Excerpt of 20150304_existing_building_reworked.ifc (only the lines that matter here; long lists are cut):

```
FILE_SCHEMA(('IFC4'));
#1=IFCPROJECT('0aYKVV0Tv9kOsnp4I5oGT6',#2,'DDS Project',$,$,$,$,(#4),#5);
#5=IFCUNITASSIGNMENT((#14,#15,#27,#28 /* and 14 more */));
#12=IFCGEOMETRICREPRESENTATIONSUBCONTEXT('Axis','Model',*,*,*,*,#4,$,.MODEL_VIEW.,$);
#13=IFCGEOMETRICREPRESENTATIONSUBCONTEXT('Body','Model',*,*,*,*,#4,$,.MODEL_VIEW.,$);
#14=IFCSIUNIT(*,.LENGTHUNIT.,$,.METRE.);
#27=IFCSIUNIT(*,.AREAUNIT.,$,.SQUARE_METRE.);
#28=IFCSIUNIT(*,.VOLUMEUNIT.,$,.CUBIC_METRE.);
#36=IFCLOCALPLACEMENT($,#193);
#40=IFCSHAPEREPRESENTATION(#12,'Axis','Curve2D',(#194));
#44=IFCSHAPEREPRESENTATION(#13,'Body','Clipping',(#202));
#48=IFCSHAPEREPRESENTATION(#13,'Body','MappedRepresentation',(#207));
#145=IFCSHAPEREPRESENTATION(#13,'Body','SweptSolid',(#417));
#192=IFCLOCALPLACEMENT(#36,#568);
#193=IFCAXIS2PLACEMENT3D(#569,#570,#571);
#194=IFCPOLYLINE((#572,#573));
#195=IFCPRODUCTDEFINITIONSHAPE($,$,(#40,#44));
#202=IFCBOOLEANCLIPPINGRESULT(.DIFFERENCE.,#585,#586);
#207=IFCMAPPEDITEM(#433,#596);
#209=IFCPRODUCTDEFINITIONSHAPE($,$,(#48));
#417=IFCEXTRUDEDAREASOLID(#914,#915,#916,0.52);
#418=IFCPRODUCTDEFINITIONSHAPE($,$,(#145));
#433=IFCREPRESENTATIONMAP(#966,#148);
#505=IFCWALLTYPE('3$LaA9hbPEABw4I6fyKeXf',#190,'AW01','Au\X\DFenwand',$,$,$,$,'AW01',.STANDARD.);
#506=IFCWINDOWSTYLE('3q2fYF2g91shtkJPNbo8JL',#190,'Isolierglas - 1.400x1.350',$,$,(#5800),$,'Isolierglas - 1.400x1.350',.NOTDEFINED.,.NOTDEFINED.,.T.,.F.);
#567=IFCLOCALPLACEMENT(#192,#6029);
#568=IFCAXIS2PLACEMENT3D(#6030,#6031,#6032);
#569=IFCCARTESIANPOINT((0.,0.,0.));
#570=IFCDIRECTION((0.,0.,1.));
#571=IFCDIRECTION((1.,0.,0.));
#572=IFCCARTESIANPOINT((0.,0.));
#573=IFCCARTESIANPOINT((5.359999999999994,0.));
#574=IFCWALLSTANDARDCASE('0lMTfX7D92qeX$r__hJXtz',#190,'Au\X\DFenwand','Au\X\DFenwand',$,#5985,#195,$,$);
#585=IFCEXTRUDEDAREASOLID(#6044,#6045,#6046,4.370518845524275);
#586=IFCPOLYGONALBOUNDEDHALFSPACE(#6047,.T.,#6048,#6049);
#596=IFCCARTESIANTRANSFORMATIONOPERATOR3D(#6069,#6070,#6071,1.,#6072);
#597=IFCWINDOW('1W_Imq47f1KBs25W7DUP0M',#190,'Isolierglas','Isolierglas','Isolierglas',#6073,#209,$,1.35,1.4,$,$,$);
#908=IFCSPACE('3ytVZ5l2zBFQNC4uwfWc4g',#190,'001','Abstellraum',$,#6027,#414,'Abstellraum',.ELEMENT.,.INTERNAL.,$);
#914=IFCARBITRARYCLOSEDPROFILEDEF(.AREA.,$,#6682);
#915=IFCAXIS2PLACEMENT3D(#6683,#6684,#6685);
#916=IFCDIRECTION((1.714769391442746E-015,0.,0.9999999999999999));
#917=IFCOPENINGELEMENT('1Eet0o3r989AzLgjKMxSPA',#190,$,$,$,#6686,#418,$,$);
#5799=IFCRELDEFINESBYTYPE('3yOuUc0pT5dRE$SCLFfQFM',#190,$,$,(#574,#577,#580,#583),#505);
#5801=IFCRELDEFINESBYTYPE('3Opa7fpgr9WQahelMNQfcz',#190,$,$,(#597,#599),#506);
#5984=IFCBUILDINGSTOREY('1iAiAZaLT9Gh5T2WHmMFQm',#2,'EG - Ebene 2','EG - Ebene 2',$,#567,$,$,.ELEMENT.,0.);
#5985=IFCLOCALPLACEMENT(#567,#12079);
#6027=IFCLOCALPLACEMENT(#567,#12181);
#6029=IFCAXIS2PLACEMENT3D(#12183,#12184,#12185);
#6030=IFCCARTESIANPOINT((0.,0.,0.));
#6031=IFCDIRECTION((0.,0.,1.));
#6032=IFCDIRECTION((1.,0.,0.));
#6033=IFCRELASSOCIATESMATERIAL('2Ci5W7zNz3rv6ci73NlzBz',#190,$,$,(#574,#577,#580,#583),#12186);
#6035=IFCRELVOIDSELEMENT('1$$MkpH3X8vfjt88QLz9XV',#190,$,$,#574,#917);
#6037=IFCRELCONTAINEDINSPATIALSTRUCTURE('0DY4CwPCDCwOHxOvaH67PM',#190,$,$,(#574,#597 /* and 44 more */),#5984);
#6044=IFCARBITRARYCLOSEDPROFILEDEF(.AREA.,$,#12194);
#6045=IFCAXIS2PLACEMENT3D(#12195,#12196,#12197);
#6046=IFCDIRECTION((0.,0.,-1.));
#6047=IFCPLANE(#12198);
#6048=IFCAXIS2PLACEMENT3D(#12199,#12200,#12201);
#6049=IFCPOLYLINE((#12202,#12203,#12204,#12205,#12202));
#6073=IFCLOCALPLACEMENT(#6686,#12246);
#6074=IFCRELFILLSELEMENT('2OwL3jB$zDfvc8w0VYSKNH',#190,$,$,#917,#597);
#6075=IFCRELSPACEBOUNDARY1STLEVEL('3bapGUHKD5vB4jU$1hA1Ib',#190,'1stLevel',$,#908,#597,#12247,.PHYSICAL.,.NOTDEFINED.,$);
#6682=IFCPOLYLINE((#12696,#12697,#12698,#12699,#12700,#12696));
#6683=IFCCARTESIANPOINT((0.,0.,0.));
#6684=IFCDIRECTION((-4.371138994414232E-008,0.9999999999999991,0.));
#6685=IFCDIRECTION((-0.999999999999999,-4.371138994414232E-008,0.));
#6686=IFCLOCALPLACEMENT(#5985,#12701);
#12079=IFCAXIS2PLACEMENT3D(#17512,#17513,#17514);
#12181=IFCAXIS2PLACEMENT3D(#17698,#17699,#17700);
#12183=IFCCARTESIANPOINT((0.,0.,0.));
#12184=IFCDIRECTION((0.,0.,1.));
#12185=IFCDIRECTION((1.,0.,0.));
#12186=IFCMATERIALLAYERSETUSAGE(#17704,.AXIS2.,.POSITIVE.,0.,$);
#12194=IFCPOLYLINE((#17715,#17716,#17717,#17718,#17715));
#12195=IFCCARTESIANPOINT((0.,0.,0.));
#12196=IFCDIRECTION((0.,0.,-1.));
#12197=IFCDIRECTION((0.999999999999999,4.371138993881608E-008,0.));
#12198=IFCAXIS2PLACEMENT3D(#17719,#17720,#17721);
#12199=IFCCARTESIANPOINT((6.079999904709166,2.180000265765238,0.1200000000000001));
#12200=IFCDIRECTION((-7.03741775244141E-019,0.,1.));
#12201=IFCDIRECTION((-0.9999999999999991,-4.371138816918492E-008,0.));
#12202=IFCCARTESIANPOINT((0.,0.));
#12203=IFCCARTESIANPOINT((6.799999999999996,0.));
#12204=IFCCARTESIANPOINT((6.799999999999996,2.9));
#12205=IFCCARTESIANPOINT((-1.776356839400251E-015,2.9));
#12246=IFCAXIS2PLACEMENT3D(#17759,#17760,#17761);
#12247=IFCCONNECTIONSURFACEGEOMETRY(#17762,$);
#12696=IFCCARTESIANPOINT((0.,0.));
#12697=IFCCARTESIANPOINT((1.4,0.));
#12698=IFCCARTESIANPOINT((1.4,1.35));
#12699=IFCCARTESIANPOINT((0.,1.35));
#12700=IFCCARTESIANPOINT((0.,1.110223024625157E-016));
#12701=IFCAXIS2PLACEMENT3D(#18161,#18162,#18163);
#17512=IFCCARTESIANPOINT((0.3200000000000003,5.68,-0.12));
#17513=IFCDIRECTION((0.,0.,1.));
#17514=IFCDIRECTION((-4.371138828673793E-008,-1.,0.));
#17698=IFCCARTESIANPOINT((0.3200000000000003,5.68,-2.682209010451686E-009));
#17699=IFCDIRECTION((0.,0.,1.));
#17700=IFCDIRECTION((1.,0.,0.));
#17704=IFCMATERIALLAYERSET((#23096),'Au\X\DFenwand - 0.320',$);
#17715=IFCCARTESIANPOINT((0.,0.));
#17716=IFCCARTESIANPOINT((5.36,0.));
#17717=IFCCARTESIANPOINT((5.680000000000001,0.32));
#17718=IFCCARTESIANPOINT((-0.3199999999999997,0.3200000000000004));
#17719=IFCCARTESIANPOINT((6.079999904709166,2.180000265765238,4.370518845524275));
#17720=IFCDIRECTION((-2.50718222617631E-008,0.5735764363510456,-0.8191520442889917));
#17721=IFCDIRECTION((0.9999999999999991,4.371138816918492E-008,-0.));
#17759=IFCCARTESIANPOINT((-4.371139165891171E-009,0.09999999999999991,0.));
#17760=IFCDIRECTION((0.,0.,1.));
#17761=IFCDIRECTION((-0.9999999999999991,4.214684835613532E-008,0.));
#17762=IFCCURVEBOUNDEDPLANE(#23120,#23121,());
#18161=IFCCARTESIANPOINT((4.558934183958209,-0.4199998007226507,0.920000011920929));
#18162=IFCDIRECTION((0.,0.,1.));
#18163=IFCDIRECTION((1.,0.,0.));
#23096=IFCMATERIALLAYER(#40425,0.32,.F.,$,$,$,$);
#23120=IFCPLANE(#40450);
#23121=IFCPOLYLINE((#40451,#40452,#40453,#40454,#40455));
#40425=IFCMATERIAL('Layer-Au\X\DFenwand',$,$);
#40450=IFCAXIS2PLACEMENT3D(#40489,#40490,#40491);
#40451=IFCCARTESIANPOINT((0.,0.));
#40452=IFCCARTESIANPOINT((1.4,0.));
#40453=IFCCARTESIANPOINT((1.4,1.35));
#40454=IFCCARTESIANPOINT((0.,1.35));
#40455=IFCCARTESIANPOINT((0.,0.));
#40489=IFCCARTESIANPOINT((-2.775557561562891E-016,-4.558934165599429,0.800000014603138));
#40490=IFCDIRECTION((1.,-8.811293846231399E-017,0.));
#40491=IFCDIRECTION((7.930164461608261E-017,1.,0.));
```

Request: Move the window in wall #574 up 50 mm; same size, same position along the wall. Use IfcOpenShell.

```python
import numpy as np
import ifcopenshell
import ifcopenshell.api.geometry
import ifcopenshell.util.placement
import ifcopenshell.util.unit

model = ifcopenshell.open("20150304_existing_building_reworked.ifc")
unit_scale = ifcopenshell.util.unit.calculate_unit_scale(model)

window = model.by_guid("1W_Imq47f1KBs25W7DUP0M")
opening = window.FillsVoids[0].RelatingOpeningElement
dz = 0.05 / unit_scale

shift = np.array([0.0, 0.0, dz])
# The window is placed relative to its opening, so it follows when the opening moves.
matrix = ifcopenshell.util.placement.get_local_placement(opening.ObjectPlacement)
matrix[:3, 3] += shift
ifcopenshell.api.geometry.edit_object_placement(
    model, product=opening, matrix=matrix, is_si=False, should_transform_children=True
)

# Space boundary surfaces are stored in each space's coordinates; move them too.
for rel in window.ProvidesBoundaries:
    if not rel.ConnectionGeometry:
        continue
    surface = rel.ConnectionGeometry.SurfaceOnRelatingElement.BasisSurface
    space_matrix = ifcopenshell.util.placement.get_local_placement(rel.RelatingSpace.ObjectPlacement)
    point = np.array(surface.Position.Location.Coordinates) + space_matrix[:3, :3].T @ shift
    surface.Position = model.createIfcAxis2Placement3D(
        model.createIfcCartesianPoint(point.tolist()), surface.Position.Axis, surface.Position.RefDirection
    )

print(f"moved by {dz * unit_scale:+.3f} m")

model.write("20150304_existing_building_reworked_rev.ifc")
```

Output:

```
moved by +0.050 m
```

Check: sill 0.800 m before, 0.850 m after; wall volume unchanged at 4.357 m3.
